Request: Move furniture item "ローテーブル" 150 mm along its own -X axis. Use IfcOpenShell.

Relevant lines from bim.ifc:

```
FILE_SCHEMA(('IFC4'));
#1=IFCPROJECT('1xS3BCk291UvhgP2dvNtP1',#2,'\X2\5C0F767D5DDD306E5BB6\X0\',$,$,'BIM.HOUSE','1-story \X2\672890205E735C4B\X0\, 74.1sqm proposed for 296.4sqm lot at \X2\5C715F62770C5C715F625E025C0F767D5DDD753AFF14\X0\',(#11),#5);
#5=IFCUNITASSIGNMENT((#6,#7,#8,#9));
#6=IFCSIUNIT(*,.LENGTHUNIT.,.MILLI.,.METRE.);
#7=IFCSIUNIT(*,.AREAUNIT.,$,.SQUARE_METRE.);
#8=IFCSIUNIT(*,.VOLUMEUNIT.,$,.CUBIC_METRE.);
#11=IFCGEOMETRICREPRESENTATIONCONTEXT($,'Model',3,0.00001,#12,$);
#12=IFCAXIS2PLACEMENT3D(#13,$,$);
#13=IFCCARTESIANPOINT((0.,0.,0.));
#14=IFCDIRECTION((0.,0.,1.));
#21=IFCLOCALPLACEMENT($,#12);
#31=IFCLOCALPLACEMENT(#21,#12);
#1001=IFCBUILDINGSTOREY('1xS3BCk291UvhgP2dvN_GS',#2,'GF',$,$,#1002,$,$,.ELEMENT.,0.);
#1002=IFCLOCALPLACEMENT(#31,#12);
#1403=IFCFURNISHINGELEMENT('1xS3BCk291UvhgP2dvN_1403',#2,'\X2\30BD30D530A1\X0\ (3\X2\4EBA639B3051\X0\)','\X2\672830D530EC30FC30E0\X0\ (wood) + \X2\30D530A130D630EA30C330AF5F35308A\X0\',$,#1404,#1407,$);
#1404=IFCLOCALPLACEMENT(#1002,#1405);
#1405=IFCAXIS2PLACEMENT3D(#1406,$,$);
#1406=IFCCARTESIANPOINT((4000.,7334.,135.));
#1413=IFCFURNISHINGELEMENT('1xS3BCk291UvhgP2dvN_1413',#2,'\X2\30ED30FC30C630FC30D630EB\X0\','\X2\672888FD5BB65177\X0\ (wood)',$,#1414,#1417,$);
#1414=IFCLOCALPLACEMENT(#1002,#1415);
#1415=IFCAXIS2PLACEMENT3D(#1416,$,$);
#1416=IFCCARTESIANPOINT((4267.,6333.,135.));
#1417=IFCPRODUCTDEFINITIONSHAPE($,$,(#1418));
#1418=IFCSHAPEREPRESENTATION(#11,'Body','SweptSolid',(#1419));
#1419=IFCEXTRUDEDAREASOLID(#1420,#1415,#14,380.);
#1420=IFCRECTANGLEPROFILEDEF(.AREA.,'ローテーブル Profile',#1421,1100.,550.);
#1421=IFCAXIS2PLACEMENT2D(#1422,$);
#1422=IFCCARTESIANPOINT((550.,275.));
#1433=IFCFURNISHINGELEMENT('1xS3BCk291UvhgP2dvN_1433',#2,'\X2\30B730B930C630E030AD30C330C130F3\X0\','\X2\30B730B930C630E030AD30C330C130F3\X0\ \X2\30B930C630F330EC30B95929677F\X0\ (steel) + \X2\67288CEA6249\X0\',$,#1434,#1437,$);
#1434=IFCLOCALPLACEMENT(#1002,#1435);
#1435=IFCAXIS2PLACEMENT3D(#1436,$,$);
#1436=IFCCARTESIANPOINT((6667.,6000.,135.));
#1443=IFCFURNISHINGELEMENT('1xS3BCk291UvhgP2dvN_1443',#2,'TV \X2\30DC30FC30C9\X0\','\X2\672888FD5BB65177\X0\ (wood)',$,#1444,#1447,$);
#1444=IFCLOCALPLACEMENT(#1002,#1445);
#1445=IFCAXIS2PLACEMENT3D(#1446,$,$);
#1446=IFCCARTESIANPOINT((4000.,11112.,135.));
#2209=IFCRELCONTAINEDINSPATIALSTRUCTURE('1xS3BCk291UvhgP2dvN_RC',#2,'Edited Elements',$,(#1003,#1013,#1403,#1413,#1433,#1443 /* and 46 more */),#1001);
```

```python
import ifcopenshell
import ifcopenshell.api.geometry
import ifcopenshell.util.placement

model = ifcopenshell.open("bim.ifc")

item = model.by_guid("1xS3BCk291UvhgP2dvN_1413")
matrix = ifcopenshell.util.placement.get_local_placement(item.ObjectPlacement)
matrix[:3, 3] -= matrix[:3, 0] * 150.0
ifcopenshell.api.geometry.edit_object_placement(model, product=item, matrix=matrix, is_si=False)

print(ifcopenshell.util.placement.get_local_placement(item.ObjectPlacement).round(3) + 0.0)

model.write("bim_v2.ifc")
```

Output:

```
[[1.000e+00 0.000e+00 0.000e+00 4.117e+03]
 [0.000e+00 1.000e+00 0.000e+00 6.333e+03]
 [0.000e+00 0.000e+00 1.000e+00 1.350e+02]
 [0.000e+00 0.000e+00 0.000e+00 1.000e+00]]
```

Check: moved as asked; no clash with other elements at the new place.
